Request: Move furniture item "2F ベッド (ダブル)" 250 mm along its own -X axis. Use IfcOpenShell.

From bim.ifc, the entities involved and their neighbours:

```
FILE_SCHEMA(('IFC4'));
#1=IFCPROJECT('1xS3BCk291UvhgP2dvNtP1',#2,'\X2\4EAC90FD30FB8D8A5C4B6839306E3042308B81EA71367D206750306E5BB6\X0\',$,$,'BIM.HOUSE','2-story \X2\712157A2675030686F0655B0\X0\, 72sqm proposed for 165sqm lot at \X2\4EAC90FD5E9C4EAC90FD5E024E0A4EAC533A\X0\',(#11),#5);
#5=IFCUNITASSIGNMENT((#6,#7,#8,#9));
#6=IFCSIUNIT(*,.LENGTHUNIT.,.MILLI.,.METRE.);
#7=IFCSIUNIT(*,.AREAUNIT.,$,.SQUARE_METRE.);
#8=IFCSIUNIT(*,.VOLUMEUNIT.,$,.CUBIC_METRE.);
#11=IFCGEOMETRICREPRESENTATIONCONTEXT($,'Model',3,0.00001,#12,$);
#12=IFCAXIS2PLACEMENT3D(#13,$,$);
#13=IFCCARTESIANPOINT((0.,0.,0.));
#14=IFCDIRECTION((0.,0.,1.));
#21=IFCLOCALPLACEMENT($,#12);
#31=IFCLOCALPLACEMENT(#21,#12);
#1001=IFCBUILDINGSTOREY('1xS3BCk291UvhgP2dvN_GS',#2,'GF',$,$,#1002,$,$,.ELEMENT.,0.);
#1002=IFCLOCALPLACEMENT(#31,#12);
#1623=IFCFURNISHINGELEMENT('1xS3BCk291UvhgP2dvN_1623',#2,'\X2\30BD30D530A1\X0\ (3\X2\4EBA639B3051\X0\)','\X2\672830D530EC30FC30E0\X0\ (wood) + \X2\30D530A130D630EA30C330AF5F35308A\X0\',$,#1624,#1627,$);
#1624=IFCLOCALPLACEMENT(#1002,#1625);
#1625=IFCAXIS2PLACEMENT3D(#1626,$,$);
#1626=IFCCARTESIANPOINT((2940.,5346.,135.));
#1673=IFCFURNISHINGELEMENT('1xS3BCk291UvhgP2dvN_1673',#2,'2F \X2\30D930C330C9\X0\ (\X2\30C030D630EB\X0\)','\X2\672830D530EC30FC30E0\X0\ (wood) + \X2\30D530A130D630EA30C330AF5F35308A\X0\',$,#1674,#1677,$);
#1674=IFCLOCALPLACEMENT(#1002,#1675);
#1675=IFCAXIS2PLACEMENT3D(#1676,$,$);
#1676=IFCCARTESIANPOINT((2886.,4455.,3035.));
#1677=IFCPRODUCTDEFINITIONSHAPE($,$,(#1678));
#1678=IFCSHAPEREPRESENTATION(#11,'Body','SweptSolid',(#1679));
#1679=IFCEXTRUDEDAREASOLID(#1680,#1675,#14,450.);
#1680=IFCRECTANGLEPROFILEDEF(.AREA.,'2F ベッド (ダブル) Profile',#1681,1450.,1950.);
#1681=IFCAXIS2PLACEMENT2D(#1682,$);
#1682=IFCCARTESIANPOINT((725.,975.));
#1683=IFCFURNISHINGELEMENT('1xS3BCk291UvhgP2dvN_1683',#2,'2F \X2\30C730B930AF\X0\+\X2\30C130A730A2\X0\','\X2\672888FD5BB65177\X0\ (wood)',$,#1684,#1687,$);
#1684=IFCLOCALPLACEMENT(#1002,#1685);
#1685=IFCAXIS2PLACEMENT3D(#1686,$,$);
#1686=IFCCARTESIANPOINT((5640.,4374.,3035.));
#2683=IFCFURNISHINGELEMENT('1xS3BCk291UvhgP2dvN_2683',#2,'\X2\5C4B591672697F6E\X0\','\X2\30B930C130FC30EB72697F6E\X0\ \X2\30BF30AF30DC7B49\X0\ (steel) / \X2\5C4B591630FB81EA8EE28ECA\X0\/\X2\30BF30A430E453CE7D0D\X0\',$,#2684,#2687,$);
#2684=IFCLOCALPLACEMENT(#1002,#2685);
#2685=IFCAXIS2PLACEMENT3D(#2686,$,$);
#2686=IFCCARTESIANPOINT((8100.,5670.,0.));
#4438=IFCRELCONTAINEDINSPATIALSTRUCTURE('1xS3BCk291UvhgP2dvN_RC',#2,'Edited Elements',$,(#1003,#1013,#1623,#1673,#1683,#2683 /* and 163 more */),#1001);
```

```python
import ifcopenshell
import ifcopenshell.api.geometry
import ifcopenshell.util.placement
import ifcopenshell.util.unit

model = ifcopenshell.open("bim.ifc")
unit_scale = ifcopenshell.util.unit.calculate_unit_scale(model)

item = model.by_id(1673)
matrix = ifcopenshell.util.placement.get_local_placement(item.ObjectPlacement)
matrix[:3, 3] -= matrix[:3, 0] * 0.25 / unit_scale
ifcopenshell.api.geometry.edit_object_placement(model, product=item, matrix=matrix, is_si=False)

print(ifcopenshell.util.placement.get_local_placement(item.ObjectPlacement).round(3) + 0.0)

model.write("bim-out.ifc")
```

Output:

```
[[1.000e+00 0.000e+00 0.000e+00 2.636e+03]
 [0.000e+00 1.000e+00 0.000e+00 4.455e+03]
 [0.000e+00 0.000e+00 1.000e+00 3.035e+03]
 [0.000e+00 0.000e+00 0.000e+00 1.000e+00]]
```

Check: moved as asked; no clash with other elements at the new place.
